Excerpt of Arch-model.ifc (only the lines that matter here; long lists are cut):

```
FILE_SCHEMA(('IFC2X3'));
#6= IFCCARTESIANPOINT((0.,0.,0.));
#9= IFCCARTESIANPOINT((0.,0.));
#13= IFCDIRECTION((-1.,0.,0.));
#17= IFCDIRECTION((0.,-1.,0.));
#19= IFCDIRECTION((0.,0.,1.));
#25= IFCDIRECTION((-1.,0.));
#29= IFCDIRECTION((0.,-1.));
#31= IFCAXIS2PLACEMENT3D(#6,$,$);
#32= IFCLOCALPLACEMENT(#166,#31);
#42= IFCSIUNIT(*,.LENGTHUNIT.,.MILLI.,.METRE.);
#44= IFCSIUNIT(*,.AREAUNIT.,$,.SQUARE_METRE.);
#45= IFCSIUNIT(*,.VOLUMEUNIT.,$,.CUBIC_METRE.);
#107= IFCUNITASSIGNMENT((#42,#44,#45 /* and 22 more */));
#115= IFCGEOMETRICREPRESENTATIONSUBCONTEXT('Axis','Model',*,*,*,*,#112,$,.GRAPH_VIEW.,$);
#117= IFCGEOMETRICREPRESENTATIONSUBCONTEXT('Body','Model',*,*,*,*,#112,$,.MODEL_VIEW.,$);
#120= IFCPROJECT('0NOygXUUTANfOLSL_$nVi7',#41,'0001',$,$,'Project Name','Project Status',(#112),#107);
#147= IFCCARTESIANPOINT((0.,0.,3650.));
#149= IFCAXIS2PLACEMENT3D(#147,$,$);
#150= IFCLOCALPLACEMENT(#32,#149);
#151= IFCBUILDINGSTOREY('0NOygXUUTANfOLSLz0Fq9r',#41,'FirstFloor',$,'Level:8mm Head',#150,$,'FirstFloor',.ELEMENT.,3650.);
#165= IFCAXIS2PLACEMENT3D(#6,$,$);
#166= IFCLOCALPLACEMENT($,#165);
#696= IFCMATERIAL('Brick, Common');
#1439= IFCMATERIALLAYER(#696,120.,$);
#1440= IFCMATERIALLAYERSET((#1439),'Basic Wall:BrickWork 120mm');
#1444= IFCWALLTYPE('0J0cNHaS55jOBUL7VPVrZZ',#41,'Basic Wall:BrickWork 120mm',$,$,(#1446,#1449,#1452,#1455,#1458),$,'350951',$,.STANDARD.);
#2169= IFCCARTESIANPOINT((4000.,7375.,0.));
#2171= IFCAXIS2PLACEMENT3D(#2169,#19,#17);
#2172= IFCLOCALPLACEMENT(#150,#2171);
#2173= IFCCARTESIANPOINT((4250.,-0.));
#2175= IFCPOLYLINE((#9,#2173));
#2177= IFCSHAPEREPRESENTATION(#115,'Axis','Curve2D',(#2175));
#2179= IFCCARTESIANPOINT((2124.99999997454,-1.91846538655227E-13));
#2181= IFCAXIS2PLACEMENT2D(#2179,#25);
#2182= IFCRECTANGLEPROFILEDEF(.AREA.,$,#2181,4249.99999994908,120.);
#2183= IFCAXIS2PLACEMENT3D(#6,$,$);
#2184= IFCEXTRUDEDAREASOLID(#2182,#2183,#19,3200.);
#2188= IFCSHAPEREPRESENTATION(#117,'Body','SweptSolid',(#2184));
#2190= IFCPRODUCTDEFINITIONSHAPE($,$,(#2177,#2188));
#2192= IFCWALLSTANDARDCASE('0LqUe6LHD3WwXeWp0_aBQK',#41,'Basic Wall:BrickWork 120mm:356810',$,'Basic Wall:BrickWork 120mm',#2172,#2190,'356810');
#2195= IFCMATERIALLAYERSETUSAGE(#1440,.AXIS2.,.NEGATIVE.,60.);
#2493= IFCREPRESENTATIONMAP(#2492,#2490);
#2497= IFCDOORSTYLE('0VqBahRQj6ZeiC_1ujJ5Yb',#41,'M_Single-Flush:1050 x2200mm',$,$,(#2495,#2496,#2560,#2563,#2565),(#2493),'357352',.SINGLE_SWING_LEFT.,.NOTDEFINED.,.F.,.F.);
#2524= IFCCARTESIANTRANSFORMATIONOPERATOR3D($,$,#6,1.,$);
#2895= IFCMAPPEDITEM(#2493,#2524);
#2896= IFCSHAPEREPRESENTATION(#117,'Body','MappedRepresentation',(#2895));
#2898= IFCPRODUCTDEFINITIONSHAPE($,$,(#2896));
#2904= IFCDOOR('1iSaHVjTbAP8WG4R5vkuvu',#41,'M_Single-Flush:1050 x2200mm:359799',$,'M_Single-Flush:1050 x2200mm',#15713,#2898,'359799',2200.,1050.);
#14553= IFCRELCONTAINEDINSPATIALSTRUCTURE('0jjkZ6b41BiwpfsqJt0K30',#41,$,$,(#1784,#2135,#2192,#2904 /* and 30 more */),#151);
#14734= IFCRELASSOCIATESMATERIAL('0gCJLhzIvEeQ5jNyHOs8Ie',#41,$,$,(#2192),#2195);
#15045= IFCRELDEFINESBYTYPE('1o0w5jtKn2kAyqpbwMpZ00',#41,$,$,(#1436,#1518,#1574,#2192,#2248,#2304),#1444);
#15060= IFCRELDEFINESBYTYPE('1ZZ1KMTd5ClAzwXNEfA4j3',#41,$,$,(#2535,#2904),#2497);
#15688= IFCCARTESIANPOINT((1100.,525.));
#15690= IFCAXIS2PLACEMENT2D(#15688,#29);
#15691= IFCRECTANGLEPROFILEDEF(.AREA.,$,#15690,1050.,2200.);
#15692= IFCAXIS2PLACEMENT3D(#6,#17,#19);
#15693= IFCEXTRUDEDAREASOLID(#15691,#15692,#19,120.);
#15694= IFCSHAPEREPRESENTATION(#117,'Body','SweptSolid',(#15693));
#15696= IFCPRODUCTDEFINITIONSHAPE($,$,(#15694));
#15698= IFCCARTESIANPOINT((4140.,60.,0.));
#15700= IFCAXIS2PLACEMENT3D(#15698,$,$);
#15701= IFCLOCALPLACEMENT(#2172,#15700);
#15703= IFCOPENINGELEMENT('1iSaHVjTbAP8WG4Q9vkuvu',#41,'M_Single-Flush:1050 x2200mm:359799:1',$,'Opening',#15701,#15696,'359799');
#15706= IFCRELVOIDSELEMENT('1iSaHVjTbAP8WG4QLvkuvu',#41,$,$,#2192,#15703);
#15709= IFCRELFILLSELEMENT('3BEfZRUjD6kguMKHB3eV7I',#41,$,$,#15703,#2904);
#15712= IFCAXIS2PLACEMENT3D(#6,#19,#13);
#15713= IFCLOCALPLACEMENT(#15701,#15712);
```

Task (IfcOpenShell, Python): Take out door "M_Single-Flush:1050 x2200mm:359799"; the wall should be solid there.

```python
import ifcopenshell
import ifcopenshell.api.feature
import ifcopenshell.api.root
import ifcopenshell.geom
import ifcopenshell.util.shape

model = ifcopenshell.open("Arch-model.ifc")
settings = ifcopenshell.geom.settings()


def volume(element):
    """Net volume in cubic metres, openings subtracted."""
    shape = ifcopenshell.geom.create_shape(settings, element)
    return ifcopenshell.util.shape.get_volume(shape.geometry)


door = model.by_guid("1iSaHVjTbAP8WG4R5vkuvu")
opening = door.FillsVoids[0].RelatingOpeningElement
wall = opening.VoidsElements[0].RelatingBuildingElement
before = volume(wall)

ifcopenshell.api.root.remove_product(model, product=door)
ifcopenshell.api.feature.remove_feature(model, feature=opening)

after = volume(wall)

print(f"wall volume {before:.3f} -> {after:.3f} m3")

model.write("Arch-model_rev.ifc")
```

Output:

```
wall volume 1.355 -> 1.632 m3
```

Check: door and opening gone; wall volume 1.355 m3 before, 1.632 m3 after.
